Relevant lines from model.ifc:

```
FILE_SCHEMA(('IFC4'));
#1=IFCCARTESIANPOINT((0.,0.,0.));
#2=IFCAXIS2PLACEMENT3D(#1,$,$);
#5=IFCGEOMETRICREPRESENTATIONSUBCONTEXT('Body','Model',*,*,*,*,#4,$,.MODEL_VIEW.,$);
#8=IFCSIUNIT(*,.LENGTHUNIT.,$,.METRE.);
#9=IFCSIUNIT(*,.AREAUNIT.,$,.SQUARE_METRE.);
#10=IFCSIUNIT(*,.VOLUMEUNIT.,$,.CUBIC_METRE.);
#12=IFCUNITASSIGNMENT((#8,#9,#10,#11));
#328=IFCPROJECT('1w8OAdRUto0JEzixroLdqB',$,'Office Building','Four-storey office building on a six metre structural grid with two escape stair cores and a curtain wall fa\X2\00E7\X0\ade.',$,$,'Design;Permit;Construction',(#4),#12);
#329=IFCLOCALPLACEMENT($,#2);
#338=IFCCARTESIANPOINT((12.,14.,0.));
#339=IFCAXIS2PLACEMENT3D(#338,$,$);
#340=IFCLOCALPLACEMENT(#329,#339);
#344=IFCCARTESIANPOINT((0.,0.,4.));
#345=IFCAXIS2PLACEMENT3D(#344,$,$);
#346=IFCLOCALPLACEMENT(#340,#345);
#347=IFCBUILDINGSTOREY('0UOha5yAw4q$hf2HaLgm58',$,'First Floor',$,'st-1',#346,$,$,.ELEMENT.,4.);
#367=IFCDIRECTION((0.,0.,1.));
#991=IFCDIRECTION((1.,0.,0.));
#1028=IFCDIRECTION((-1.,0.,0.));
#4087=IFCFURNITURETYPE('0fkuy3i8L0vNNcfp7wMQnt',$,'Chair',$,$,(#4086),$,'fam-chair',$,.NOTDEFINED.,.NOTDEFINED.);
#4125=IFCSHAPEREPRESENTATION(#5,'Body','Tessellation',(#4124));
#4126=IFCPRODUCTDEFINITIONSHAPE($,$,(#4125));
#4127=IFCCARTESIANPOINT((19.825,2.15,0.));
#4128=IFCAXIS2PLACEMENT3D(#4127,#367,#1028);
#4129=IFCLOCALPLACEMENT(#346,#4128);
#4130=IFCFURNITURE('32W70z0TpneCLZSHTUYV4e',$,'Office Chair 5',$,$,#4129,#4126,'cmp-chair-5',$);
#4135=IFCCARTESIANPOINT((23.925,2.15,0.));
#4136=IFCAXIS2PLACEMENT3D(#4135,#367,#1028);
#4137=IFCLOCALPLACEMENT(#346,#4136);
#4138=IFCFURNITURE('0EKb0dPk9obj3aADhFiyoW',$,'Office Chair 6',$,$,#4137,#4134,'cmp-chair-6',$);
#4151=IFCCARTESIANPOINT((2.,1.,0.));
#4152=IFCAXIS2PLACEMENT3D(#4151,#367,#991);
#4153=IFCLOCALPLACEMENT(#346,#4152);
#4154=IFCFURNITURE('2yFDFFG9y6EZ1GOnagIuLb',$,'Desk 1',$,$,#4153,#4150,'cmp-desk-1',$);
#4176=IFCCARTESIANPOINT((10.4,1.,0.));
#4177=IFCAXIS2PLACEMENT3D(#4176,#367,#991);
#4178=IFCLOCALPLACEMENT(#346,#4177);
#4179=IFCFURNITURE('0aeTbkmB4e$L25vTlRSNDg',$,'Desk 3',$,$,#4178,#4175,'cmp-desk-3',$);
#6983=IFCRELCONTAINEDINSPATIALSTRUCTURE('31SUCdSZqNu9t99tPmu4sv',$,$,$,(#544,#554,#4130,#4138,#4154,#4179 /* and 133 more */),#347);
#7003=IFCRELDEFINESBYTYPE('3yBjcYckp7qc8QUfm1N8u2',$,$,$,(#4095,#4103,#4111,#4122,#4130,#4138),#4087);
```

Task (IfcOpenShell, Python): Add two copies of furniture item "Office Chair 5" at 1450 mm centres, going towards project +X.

```python
import numpy as np
import ifcopenshell
import ifcopenshell.api.geometry
import ifcopenshell.api.root
import ifcopenshell.util.element
import ifcopenshell.util.placement
import ifcopenshell.util.unit

model = ifcopenshell.open("model.ifc")
unit_scale = ifcopenshell.util.unit.calculate_unit_scale(model)

source = model.by_guid("32W70z0TpneCLZSHTUYV4e")
base = ifcopenshell.util.placement.get_local_placement(source.ObjectPlacement)
step = np.array([1.0, 0.0, 0.0]) * 1.45 / unit_scale

for i in range(1, 3):
    copy = ifcopenshell.api.root.copy_class(model, product=source)
    copy.Representation = ifcopenshell.util.element.copy_deep(
        model, source.Representation, exclude=["IfcGeometricRepresentationContext", "IfcRepresentationMap"]
    )
    copy.Tag = None
    matrix = base.copy()
    matrix[:3, 3] += i * step
    print("added at", matrix[:3, 3].round(3) + 0.0)
    ifcopenshell.api.geometry.edit_object_placement(model, product=copy, matrix=matrix, is_si=False)

model.write("model_updated.ifc")
```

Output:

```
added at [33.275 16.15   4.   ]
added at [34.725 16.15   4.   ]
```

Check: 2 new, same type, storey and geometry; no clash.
